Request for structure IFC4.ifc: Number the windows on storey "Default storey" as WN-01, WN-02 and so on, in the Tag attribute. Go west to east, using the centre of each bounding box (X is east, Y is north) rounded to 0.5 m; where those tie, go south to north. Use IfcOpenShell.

First a look at what the model holds.

```python
import ifcopenshell
import ifcopenshell.util.element
import ifcopenshell.util.placement

model = ifcopenshell.open("structure IFC4.ifc")
print(model.schema)
storey = next(s for s in model.by_type("IfcBuildingStorey") if s.Name == "Default storey")
windows = [e for e in ifcopenshell.util.element.get_decomposition(storey) if e.is_a("IfcWindow")]
for e in sorted(windows, key=lambda e: e.id()):
    origin = ifcopenshell.util.placement.get_local_placement(e.ObjectPlacement)[:3, 3]
    print(e.id(), e.Tag, e.Name, origin.round(2) + 0.0, sep=" | ")
```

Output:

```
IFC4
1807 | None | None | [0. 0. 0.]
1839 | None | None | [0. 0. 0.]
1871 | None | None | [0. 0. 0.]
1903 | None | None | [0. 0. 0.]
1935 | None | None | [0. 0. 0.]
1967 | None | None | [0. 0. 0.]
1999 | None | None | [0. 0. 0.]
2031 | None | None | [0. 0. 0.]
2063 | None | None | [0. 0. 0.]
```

```python
import ifcopenshell
import ifcopenshell.geom
import ifcopenshell.util.element
import ifcopenshell.util.shape

model = ifcopenshell.open("structure IFC4.ifc")
settings = ifcopenshell.geom.settings()
settings.set("use-world-coords", True)


def centre(element):
    shape = ifcopenshell.geom.create_shape(settings, element)
    return ifcopenshell.util.shape.get_bbox_centroid(shape.geometry)


storey = next(s for s in model.by_type("IfcBuildingStorey") if s.Name == "Default storey")
windows = [e for e in ifcopenshell.util.element.get_decomposition(storey) if e.is_a("IfcWindow")]

# Insertion points can sit at a corner or the storey origin, so sort by the geometry (in metres).
centres = {e: centre(e) for e in windows}
windows.sort(key=lambda e: (round(centres[e][0] / 0.5), centres[e][1]))

for i, e in enumerate(windows, start=1):
    number = f"WN-{i:02d}"
    e.Tag = number
    print(e.id(), number)

model.write("structure IFC4-out.ifc")
```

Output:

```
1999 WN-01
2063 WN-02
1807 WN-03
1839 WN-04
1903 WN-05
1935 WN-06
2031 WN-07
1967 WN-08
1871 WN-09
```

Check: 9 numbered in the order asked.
